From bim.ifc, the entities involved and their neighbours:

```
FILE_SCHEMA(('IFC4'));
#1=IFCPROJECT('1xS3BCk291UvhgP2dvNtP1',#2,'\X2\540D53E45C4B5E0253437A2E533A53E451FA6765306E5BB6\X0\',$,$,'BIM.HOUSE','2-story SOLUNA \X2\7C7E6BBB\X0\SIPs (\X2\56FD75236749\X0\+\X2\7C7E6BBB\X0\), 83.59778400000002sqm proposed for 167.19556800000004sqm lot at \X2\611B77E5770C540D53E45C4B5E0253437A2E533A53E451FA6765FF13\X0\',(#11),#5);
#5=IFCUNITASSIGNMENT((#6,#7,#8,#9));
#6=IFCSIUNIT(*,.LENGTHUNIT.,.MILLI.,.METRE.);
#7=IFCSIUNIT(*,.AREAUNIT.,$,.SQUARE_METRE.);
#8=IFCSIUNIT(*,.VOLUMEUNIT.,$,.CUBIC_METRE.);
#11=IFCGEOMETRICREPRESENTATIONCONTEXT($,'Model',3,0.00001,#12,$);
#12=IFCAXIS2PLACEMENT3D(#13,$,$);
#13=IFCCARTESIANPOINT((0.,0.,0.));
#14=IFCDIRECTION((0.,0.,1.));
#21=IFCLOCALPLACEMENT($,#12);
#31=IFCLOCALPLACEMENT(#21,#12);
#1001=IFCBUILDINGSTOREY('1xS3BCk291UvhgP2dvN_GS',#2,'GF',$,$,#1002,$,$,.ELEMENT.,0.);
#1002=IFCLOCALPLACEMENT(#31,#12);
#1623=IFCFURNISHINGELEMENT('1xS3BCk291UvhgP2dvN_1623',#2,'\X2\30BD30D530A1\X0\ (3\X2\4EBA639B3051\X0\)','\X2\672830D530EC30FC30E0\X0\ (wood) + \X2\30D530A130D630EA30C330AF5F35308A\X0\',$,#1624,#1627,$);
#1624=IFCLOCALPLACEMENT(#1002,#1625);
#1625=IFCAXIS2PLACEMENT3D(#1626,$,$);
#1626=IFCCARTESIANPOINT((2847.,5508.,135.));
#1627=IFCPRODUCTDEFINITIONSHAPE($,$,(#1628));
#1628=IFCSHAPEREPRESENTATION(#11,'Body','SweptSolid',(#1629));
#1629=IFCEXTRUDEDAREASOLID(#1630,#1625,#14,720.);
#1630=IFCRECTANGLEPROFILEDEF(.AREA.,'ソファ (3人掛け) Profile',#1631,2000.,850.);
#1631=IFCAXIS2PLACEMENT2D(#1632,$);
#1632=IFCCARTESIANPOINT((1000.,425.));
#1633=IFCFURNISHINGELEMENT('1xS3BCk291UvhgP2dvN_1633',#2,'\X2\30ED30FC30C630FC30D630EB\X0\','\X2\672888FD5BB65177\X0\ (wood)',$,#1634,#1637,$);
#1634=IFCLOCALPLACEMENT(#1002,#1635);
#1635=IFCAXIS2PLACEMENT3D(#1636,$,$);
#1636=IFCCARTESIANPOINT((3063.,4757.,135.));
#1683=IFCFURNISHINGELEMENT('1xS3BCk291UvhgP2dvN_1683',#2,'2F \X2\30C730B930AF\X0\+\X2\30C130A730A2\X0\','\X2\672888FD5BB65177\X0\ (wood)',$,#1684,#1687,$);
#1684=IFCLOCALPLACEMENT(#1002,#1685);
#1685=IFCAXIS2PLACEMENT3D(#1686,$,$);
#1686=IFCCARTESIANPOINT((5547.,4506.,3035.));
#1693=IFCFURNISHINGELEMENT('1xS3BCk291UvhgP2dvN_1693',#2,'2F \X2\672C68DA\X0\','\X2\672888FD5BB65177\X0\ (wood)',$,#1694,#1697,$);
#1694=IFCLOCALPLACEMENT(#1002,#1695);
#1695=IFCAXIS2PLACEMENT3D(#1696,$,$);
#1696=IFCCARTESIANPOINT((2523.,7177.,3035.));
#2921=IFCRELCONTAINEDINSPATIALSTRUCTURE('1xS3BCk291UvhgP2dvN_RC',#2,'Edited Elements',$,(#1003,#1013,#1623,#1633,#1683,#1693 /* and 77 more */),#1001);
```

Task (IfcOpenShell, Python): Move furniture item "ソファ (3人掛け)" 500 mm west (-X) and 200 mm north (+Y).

```python
import ifcopenshell
import ifcopenshell.api.geometry
import ifcopenshell.util.placement
import ifcopenshell.util.unit

model = ifcopenshell.open("bim.ifc")
unit_scale = ifcopenshell.util.unit.calculate_unit_scale(model)

item = model.by_guid("1xS3BCk291UvhgP2dvN_1623")
matrix = ifcopenshell.util.placement.get_local_placement(item.ObjectPlacement)
matrix[0, 3] -= 0.5 / unit_scale
matrix[1, 3] += 0.2 / unit_scale
ifcopenshell.api.geometry.edit_object_placement(model, product=item, matrix=matrix, is_si=False)

print(ifcopenshell.util.placement.get_local_placement(item.ObjectPlacement).round(3) + 0.0)

model.write("bim_rev.ifc")
```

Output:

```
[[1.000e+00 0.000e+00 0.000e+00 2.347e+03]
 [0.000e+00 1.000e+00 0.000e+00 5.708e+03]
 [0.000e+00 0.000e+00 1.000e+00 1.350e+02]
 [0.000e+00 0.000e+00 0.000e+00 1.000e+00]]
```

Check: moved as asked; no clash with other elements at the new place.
